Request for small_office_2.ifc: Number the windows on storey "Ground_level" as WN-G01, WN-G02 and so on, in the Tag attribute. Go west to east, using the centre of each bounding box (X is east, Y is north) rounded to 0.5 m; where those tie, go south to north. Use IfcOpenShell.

First a look at what the model holds.

```python
import ifcopenshell
import ifcopenshell.util.element
import ifcopenshell.util.placement

model = ifcopenshell.open("small_office_2.ifc")
print(model.schema)
storey = next(s for s in model.by_type("IfcBuildingStorey") if s.Name == "Ground_level")
windows = [e for e in ifcopenshell.util.element.get_decomposition(storey) if e.is_a("IfcWindow")]
for e in sorted(windows, key=lambda e: e.id()):
    origin = ifcopenshell.util.placement.get_local_placement(e.ObjectPlacement)[:3, 3]
    print(e.id(), e.Tag, e.Name, origin.round(2) + 0.0, sep=" | ")
```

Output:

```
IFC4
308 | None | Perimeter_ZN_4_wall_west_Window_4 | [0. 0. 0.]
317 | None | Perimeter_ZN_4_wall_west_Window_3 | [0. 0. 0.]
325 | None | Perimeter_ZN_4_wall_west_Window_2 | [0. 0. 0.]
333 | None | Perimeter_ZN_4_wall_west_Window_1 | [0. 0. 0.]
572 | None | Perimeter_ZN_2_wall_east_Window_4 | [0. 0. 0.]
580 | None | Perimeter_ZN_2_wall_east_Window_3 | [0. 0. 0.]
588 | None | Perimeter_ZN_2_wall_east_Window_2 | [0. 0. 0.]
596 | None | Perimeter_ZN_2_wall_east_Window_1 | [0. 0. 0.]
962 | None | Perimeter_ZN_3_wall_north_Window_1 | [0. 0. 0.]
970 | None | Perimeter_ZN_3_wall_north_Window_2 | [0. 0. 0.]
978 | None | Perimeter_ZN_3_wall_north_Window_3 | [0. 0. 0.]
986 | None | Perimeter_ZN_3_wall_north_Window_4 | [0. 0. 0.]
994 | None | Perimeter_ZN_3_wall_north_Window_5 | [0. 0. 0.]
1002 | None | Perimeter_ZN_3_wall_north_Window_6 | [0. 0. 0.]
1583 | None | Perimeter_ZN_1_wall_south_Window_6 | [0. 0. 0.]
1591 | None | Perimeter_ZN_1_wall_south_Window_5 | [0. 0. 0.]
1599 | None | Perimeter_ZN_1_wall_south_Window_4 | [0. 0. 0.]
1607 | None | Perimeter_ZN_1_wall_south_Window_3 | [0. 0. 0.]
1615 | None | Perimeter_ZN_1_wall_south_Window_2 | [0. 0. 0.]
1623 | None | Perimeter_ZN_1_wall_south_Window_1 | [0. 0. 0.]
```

```python
import ifcopenshell
import ifcopenshell.geom
import ifcopenshell.util.element
import ifcopenshell.util.shape

model = ifcopenshell.open("small_office_2.ifc")
settings = ifcopenshell.geom.settings()
settings.set("use-world-coords", True)


def centre(element):
    shape = ifcopenshell.geom.create_shape(settings, element)
    return ifcopenshell.util.shape.get_bbox_centroid(shape.geometry)


storey = next(s for s in model.by_type("IfcBuildingStorey") if s.Name == "Ground_level")
windows = [e for e in ifcopenshell.util.element.get_decomposition(storey) if e.is_a("IfcWindow")]

# Insertion points can sit at a corner or the storey origin, so sort by the geometry (in metres).
centres = {e: centre(e) for e in windows}
windows.sort(key=lambda e: (round(centres[e][0] / 0.5), centres[e][1]))

for i, e in enumerate(windows, start=1):
    number = f"WN-G{i:02d}"
    e.Tag = number
    print(e.id(), number)

model.write("small_office_2_v2.ifc")
```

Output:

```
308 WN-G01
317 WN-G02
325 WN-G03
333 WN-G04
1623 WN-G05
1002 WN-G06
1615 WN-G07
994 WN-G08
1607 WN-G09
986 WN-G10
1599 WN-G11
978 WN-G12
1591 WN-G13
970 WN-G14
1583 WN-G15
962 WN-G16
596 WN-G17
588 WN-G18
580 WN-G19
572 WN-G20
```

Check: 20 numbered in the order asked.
